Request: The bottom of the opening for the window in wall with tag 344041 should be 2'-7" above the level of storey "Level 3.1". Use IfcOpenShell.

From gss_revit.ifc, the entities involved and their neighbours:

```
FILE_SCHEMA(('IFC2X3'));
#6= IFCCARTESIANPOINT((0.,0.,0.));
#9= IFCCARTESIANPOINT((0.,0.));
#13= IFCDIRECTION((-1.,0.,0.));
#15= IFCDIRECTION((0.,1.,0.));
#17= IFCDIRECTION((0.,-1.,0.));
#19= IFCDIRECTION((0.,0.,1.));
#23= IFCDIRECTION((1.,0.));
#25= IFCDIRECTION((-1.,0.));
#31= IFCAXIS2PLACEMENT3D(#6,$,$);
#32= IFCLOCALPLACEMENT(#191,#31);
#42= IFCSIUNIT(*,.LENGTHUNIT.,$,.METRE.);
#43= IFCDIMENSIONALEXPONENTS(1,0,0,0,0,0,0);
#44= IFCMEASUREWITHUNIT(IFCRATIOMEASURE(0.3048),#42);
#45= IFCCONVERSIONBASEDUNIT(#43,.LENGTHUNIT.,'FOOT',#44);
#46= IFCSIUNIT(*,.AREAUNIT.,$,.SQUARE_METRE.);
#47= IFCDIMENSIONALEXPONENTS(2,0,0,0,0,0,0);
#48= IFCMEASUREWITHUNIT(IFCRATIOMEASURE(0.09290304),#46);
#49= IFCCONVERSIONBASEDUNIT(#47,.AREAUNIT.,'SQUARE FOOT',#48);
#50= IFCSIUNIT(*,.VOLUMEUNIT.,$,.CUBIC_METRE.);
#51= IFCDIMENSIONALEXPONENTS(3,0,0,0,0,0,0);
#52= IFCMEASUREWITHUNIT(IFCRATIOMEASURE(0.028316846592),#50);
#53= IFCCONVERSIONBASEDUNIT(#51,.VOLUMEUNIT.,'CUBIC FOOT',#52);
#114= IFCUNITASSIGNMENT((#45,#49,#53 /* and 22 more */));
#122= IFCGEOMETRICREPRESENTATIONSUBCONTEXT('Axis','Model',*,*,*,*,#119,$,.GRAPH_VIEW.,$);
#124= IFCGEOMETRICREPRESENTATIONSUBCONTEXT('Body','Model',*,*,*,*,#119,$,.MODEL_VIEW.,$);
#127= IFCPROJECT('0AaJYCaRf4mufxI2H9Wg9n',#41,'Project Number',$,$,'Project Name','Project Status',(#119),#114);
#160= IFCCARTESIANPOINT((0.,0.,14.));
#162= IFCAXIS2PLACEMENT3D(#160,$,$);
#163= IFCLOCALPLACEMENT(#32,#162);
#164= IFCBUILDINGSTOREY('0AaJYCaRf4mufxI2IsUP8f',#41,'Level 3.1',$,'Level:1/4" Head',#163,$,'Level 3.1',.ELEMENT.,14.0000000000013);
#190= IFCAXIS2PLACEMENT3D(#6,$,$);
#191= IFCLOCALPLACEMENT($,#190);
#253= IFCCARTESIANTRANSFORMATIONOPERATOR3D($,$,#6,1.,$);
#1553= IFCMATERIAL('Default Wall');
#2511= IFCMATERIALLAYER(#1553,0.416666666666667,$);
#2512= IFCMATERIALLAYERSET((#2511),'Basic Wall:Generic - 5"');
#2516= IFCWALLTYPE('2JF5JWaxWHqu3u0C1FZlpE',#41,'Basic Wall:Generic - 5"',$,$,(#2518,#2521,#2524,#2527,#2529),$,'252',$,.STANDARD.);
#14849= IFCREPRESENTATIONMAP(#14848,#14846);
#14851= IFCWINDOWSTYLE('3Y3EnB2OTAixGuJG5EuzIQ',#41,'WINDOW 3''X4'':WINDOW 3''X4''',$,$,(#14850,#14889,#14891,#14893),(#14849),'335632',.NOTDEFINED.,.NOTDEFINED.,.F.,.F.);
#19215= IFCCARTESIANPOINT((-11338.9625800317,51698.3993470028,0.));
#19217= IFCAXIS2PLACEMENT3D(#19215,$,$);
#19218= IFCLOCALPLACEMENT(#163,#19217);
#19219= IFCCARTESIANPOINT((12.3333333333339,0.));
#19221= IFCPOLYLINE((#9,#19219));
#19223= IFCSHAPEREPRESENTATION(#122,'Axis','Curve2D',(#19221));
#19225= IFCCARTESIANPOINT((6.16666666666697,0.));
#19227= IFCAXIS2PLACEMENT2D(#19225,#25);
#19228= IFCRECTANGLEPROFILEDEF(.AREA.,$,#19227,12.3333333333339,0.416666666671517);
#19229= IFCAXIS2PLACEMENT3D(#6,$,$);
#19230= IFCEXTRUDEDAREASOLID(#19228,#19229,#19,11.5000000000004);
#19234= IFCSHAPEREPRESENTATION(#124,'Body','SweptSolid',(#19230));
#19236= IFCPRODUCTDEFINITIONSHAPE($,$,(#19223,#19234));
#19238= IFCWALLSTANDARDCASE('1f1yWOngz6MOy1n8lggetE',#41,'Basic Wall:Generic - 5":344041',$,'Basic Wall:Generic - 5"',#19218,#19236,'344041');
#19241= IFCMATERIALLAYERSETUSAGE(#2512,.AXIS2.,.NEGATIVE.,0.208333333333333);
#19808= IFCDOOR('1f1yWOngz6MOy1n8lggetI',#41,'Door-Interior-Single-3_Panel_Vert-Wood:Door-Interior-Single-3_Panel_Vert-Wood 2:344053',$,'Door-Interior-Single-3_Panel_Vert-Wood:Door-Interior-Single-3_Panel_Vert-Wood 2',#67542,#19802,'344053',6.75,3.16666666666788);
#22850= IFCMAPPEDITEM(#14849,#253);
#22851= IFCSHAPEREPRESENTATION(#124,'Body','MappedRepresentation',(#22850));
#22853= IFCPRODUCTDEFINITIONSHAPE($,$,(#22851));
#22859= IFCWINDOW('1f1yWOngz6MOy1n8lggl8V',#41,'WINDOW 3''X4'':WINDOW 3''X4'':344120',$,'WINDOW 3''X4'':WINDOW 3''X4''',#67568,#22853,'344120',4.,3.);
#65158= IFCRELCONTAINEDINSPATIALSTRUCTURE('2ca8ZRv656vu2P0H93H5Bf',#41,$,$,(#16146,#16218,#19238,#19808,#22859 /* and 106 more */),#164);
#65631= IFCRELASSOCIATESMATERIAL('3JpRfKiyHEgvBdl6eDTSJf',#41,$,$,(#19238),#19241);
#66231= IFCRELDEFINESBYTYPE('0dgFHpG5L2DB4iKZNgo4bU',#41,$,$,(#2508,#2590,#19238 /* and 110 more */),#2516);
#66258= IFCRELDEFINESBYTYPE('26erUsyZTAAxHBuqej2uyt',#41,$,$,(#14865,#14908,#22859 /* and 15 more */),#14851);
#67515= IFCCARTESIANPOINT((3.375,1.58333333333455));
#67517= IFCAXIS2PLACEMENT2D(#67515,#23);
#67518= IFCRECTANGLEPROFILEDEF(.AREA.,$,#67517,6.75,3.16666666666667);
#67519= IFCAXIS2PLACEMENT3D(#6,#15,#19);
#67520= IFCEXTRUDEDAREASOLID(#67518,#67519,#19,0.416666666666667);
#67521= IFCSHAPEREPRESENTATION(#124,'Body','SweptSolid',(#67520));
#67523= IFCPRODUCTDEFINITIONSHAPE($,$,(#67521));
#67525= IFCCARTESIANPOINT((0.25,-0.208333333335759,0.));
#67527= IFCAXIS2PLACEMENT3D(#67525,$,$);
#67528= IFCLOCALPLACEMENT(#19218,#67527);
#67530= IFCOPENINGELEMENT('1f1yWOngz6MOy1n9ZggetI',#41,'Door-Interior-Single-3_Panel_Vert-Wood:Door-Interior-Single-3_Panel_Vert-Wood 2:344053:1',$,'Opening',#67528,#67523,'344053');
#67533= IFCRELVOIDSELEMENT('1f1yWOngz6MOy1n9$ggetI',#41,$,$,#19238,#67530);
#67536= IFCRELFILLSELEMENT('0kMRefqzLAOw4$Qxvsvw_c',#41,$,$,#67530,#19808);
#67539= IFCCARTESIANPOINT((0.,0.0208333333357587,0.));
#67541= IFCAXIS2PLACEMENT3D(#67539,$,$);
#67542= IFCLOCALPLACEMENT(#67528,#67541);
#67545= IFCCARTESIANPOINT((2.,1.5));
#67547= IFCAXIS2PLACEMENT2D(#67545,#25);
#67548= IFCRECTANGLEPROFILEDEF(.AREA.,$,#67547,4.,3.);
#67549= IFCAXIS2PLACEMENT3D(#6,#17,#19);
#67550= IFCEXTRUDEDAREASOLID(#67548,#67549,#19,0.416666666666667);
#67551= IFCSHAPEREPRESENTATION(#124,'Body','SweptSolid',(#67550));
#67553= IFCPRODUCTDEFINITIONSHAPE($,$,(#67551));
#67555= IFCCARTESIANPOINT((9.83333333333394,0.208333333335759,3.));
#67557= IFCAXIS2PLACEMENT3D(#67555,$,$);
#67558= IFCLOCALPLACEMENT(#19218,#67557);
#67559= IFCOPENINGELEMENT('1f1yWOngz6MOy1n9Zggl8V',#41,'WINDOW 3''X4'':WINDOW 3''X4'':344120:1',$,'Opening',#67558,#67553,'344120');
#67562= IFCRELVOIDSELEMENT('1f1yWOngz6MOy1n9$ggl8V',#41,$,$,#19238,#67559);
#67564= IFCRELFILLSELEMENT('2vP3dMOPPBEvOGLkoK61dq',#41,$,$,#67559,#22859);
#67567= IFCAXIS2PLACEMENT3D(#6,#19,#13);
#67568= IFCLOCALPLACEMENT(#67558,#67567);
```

```python
import numpy as np
import ifcopenshell
import ifcopenshell.api.geometry
import ifcopenshell.geom
import ifcopenshell.util.element
import ifcopenshell.util.placement
import ifcopenshell.util.shape
import ifcopenshell.util.unit

model = ifcopenshell.open("gss_revit.ifc")
unit_scale = ifcopenshell.util.unit.calculate_unit_scale(model)

window = model.by_id(22859)
opening = window.FillsVoids[0].RelatingOpeningElement
storey = ifcopenshell.util.element.get_container(window, ifc_class="IfcBuildingStorey")
level = ifcopenshell.util.placement.get_local_placement(storey.ObjectPlacement)[2, 3]

# The opening's origin need not be at the sill, so measure its lowest point.
shape = ifcopenshell.geom.create_shape(ifcopenshell.geom.settings(), opening)
bottom = ifcopenshell.util.shape.get_shape_bottom_elevation(shape, shape.geometry) / unit_scale
dz = level + 31 * 0.0254 / unit_scale - bottom

shift = np.array([0.0, 0.0, dz])
# The window is placed relative to its opening, so it follows when the opening moves.
matrix = ifcopenshell.util.placement.get_local_placement(opening.ObjectPlacement)
matrix[:3, 3] += shift
ifcopenshell.api.geometry.edit_object_placement(
    model, product=opening, matrix=matrix, is_si=False, should_transform_children=True
)

print(f"moved by {dz * unit_scale:+.3f} m")

model.write("gss_revit-out.ifc")
```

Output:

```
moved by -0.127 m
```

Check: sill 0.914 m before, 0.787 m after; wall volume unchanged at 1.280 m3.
